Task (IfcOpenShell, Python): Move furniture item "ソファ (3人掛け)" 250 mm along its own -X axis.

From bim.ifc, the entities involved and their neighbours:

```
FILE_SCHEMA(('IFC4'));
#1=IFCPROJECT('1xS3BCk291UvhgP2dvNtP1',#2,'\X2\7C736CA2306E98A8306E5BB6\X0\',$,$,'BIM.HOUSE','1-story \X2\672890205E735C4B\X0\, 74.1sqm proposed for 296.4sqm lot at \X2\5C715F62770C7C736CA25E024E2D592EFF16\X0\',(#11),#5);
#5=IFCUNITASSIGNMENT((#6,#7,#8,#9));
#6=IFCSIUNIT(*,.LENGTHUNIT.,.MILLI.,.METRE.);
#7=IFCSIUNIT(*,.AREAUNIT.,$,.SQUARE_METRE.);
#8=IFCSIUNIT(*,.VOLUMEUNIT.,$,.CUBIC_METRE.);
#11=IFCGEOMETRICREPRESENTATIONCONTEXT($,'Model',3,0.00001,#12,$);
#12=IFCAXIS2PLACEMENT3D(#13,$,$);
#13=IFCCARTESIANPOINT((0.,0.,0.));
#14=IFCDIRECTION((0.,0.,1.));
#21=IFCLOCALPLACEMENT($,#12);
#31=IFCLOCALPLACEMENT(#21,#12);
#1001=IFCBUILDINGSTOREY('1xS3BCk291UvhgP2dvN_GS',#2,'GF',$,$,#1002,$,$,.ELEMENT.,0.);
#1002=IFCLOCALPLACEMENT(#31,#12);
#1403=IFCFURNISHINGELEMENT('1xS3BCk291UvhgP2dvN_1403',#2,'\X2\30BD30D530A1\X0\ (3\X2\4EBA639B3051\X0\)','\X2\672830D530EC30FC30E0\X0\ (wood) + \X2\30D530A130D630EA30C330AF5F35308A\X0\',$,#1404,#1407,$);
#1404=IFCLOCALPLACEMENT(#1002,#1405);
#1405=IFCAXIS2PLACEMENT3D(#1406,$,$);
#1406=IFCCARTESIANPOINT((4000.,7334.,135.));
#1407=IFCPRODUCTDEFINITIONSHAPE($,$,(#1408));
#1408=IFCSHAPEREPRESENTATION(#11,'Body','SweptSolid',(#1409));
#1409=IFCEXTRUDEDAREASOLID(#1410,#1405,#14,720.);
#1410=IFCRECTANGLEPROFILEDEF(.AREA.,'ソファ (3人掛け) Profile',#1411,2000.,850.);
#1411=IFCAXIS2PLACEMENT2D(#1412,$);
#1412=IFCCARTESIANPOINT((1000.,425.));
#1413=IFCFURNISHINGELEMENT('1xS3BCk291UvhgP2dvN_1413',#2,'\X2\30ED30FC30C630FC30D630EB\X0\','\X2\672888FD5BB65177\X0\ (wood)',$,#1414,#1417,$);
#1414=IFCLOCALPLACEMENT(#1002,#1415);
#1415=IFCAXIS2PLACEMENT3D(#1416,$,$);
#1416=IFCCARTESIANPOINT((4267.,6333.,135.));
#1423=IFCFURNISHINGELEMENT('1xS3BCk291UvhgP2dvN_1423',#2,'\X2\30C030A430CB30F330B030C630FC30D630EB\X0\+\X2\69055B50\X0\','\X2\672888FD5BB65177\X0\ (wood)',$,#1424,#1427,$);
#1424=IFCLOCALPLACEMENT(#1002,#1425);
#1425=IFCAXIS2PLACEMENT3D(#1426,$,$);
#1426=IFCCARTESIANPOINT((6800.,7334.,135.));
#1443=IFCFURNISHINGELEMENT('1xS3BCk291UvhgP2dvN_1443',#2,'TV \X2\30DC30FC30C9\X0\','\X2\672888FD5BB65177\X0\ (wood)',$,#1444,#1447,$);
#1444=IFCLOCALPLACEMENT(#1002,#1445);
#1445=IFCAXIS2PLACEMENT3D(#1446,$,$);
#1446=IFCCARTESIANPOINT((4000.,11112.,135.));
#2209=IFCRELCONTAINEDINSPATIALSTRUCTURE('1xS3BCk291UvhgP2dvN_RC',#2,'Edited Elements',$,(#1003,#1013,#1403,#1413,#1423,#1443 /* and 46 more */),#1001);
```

```python
import ifcopenshell
import ifcopenshell.api.geometry
import ifcopenshell.util.placement

model = ifcopenshell.open("bim.ifc")

item = model.by_guid("1xS3BCk291UvhgP2dvN_1403")
matrix = ifcopenshell.util.placement.get_local_placement(item.ObjectPlacement)
matrix[:3, 3] -= matrix[:3, 0] * 250.0
ifcopenshell.api.geometry.edit_object_placement(model, product=item, matrix=matrix, is_si=False)

print(ifcopenshell.util.placement.get_local_placement(item.ObjectPlacement).round(3) + 0.0)

model.write("bim_edited.ifc")
```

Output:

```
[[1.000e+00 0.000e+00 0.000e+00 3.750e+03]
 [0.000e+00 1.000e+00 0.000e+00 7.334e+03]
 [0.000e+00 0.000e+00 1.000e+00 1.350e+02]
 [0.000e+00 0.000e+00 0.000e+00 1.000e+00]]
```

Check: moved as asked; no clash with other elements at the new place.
